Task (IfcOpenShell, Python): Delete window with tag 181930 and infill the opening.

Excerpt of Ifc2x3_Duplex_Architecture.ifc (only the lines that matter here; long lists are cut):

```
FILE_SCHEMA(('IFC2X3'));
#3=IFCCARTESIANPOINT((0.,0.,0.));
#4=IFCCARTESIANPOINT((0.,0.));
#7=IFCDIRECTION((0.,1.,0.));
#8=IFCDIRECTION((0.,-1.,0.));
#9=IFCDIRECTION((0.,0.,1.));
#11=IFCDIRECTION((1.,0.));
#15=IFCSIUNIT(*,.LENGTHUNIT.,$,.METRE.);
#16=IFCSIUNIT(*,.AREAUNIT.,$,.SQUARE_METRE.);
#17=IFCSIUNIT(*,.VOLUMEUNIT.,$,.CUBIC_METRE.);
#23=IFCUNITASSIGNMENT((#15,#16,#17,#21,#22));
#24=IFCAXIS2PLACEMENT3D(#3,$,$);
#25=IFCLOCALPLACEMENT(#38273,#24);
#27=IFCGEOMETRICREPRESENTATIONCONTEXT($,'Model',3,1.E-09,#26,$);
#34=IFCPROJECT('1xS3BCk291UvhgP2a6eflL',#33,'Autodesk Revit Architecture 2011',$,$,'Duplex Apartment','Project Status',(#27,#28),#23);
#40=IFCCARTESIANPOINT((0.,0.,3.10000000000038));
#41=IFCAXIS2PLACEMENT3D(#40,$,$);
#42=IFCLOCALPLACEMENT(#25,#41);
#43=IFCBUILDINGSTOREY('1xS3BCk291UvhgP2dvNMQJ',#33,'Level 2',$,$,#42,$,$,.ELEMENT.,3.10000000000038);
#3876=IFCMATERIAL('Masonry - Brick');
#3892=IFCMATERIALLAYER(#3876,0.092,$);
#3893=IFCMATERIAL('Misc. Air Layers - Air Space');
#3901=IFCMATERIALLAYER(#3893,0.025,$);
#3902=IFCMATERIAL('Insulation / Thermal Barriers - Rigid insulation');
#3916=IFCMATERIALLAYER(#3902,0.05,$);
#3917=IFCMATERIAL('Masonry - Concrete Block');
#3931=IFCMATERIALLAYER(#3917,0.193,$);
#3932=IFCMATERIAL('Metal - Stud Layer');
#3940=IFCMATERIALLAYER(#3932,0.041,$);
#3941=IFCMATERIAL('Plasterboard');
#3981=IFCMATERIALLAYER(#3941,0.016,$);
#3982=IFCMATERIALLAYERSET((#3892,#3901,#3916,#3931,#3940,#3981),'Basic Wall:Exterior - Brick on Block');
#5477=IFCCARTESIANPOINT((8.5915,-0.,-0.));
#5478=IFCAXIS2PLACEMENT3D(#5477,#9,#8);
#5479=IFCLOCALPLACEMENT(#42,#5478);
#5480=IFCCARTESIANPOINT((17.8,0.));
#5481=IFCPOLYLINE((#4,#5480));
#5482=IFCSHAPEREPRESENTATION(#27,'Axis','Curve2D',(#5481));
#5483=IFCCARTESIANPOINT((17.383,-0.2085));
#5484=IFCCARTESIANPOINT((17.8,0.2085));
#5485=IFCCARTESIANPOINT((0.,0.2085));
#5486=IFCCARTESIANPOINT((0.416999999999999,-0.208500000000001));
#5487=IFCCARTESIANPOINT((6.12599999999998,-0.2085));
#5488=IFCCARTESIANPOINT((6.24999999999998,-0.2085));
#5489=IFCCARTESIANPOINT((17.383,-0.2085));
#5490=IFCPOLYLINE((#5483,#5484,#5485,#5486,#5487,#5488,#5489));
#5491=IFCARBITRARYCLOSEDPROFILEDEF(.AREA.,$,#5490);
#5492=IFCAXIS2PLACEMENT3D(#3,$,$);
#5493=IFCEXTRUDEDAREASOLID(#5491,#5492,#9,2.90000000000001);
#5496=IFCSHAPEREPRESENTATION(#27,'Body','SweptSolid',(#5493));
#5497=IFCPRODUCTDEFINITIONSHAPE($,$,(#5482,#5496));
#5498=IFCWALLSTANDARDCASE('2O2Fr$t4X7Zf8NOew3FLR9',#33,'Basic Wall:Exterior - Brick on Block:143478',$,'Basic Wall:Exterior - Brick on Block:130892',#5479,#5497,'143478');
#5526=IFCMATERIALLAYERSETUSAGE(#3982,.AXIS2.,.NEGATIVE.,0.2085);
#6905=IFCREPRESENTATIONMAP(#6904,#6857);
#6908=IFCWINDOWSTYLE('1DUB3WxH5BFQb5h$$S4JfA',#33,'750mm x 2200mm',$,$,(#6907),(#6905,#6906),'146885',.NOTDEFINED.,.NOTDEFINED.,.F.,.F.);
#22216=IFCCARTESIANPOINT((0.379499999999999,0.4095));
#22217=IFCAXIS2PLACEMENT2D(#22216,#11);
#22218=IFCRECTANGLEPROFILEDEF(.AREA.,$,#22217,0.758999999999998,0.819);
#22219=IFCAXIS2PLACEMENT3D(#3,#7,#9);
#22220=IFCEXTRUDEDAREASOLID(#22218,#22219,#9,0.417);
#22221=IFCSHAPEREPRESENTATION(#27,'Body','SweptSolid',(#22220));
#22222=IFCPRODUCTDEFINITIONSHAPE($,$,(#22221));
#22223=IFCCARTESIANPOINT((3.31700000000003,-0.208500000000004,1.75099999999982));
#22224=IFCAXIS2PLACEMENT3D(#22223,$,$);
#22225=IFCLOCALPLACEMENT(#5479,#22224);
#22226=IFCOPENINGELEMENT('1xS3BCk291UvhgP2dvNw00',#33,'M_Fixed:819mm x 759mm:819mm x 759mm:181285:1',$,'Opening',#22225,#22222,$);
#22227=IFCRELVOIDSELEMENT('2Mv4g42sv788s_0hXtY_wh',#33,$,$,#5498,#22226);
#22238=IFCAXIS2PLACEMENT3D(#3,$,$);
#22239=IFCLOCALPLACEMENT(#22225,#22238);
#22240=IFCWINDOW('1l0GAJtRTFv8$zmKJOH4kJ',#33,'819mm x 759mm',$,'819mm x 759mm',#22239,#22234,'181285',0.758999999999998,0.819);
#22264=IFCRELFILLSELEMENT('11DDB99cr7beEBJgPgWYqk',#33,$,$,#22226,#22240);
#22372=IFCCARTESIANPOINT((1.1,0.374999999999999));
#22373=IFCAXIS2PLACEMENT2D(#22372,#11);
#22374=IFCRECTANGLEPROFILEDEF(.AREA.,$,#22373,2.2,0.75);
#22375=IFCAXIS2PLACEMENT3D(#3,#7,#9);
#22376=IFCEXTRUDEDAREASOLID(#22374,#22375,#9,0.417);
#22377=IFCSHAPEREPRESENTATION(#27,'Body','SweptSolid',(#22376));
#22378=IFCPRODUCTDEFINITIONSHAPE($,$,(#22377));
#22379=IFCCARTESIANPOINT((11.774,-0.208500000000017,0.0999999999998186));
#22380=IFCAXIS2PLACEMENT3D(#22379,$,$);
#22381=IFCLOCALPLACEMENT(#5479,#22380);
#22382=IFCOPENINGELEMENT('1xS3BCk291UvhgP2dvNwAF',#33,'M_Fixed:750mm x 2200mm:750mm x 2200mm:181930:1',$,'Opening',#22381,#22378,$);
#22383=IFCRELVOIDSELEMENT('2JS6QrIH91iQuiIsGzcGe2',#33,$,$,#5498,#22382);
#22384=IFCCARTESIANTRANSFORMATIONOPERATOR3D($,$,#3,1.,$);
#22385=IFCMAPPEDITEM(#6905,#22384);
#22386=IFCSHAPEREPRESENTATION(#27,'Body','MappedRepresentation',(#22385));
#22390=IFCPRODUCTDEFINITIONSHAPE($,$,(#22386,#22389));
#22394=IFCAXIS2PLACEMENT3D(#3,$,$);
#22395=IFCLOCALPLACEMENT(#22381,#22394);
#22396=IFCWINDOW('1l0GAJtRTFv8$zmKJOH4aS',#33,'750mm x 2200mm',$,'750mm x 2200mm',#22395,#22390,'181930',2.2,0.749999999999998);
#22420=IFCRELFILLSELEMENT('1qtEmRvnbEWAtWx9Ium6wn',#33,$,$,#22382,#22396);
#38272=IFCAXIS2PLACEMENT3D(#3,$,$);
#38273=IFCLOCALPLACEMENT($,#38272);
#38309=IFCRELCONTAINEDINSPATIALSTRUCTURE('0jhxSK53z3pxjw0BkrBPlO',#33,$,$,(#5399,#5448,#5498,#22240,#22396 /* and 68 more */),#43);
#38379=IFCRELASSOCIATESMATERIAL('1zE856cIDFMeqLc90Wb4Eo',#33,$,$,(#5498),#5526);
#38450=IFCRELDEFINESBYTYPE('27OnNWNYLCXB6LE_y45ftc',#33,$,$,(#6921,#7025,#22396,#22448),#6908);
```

```python
import ifcopenshell
import ifcopenshell.api.feature
import ifcopenshell.api.root
import ifcopenshell.geom
import ifcopenshell.util.shape

model = ifcopenshell.open("Ifc2x3_Duplex_Architecture.ifc")
settings = ifcopenshell.geom.settings()


def volume(element):
    """Net volume in cubic metres, openings subtracted."""
    shape = ifcopenshell.geom.create_shape(settings, element)
    return ifcopenshell.util.shape.get_volume(shape.geometry)


window = model.by_id(22396)
opening = window.FillsVoids[0].RelatingOpeningElement
wall = opening.VoidsElements[0].RelatingBuildingElement
before = volume(wall)

ifcopenshell.api.root.remove_product(model, product=window)
ifcopenshell.api.feature.remove_feature(model, feature=opening)

after = volume(wall)

print(f"wall volume {before:.3f} -> {after:.3f} m3")

model.write("Ifc2x3_Duplex_Architecture_rev.ifc")
```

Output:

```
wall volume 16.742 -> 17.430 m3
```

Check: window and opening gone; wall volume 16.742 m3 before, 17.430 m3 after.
